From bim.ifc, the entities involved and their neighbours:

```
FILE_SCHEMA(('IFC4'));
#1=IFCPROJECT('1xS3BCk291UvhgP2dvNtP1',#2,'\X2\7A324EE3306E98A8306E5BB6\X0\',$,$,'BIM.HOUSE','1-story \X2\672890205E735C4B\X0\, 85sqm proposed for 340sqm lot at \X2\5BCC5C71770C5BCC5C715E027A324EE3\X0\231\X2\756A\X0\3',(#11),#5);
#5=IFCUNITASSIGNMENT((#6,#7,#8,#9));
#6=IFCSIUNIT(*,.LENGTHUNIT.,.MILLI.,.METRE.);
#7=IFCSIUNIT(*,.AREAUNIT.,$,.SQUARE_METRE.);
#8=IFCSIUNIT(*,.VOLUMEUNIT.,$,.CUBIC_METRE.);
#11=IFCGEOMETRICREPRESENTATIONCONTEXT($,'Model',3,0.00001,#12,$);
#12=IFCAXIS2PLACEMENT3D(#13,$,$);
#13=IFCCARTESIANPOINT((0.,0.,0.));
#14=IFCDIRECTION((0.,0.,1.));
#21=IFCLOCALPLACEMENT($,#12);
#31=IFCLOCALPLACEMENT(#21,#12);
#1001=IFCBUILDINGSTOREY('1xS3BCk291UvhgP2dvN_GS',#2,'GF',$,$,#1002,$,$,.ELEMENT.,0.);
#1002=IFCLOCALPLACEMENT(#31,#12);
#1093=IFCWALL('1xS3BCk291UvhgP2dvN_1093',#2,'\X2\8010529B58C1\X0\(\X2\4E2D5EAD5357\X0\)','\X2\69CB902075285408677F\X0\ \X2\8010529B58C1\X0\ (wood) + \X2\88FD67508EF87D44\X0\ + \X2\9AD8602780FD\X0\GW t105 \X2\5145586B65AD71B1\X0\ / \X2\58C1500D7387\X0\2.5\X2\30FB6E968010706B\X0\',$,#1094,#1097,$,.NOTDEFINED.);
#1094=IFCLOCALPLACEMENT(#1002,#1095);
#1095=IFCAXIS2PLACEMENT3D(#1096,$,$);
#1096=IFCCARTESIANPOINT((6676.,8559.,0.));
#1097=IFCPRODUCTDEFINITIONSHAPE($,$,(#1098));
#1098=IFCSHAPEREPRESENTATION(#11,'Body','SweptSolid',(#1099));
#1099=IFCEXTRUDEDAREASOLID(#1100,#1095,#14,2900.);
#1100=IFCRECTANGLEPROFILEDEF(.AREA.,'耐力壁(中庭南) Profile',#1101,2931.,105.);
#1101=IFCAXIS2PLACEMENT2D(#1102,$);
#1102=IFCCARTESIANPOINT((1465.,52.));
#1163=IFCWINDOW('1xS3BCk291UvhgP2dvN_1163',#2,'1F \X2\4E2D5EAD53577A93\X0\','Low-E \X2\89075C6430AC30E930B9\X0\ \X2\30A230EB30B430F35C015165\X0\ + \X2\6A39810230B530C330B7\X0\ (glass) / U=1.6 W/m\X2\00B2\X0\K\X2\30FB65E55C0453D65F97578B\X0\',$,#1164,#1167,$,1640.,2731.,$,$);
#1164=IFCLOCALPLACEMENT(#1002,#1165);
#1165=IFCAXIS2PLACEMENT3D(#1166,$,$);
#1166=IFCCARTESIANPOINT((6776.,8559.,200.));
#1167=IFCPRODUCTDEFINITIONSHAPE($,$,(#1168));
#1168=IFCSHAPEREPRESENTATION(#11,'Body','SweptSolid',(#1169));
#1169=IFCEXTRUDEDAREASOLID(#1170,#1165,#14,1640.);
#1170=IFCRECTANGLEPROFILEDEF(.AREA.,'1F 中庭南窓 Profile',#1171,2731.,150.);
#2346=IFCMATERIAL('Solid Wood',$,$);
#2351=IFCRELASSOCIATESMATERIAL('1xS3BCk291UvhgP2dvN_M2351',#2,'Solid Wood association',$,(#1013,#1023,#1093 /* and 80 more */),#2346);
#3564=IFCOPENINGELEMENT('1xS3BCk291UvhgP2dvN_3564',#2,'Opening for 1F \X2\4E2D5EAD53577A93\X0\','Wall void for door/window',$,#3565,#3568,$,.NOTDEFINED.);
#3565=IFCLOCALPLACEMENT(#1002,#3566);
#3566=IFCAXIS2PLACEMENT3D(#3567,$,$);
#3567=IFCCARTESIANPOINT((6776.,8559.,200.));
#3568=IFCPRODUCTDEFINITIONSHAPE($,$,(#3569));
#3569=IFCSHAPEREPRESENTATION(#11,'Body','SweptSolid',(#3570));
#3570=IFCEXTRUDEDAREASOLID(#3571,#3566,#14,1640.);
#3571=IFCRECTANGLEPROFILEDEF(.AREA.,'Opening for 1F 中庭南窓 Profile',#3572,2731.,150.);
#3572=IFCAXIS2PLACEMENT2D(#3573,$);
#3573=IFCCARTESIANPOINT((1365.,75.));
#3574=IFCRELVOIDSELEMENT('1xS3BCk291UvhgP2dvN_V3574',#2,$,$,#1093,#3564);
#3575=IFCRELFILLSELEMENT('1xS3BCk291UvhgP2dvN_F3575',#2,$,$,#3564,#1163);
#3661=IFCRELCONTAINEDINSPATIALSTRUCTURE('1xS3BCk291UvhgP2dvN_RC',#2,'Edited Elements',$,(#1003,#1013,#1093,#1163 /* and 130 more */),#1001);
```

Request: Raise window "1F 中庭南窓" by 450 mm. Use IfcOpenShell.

```python
import numpy as np
import ifcopenshell
import ifcopenshell.api.geometry
import ifcopenshell.util.placement
import ifcopenshell.util.unit

model = ifcopenshell.open("bim.ifc")
unit_scale = ifcopenshell.util.unit.calculate_unit_scale(model)

window = model.by_id(1163)
opening = window.FillsVoids[0].RelatingOpeningElement
dz = 0.45 / unit_scale

shift = np.array([0.0, 0.0, dz])
# The window is not placed relative to its opening, so move both.
for product in (opening, window):
    matrix = ifcopenshell.util.placement.get_local_placement(product.ObjectPlacement)
    matrix[:3, 3] += shift
    ifcopenshell.api.geometry.edit_object_placement(model, product=product, matrix=matrix, is_si=False)

print(f"moved by {dz * unit_scale:+.3f} m")

model.write("bim_rev.ifc")
```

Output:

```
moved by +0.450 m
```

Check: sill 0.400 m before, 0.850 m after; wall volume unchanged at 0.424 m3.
